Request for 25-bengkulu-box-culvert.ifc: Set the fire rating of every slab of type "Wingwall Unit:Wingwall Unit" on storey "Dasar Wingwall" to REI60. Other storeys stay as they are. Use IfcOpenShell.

First a look at what the model holds.

```python
import ifcopenshell
import ifcopenshell.util.element

model = ifcopenshell.open("25-bengkulu-box-culvert.ifc")
print(model.schema)
storey = next(s for s in model.by_type("IfcBuildingStorey") if s.Name == "Dasar Wingwall")
slabs = [e for e in ifcopenshell.util.element.get_decomposition(storey) if e.is_a("IfcSlab")]
seen = {}
for e in slabs:
    element_type = ifcopenshell.util.element.get_type(e)
    key = (element_type.Name if element_type != e and element_type else None, ifcopenshell.util.element.get_pset(e, "Pset_SlabCommon", "FireRating"))
    seen[key] = seen.get(key, 0) + 1
for (name, value), count in sorted(seen.items(), key=str):
    print(count, "x", name, "|", value)
```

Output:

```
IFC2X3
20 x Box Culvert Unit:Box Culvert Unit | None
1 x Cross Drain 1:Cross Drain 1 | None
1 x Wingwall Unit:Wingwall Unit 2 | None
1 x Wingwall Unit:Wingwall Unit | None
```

```python
import ifcopenshell
import ifcopenshell.api.pset
import ifcopenshell.util.element

model = ifcopenshell.open("25-bengkulu-box-culvert.ifc")

storey = next(s for s in model.by_type("IfcBuildingStorey") if s.Name == "Dasar Wingwall")
slabs = [e for e in ifcopenshell.util.element.get_decomposition(storey) if e.is_a("IfcSlab")]

count = 0
for e in slabs:
    element_type = ifcopenshell.util.element.get_type(e)
    if element_type in (None, e) or element_type.Name != "Wingwall Unit:Wingwall Unit":
        continue
    # add_pset returns the element's existing set when there is one.
    pset = ifcopenshell.api.pset.add_pset(model, product=e, name="Pset_SlabCommon")
    ifcopenshell.api.pset.edit_pset(model, pset=pset, properties={"FireRating": "REI60"})
    count += 1

print(count, "slabs updated")

model.write("25-bengkulu-box-culvert_v2.ifc")
```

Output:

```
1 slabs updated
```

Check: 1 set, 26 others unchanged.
